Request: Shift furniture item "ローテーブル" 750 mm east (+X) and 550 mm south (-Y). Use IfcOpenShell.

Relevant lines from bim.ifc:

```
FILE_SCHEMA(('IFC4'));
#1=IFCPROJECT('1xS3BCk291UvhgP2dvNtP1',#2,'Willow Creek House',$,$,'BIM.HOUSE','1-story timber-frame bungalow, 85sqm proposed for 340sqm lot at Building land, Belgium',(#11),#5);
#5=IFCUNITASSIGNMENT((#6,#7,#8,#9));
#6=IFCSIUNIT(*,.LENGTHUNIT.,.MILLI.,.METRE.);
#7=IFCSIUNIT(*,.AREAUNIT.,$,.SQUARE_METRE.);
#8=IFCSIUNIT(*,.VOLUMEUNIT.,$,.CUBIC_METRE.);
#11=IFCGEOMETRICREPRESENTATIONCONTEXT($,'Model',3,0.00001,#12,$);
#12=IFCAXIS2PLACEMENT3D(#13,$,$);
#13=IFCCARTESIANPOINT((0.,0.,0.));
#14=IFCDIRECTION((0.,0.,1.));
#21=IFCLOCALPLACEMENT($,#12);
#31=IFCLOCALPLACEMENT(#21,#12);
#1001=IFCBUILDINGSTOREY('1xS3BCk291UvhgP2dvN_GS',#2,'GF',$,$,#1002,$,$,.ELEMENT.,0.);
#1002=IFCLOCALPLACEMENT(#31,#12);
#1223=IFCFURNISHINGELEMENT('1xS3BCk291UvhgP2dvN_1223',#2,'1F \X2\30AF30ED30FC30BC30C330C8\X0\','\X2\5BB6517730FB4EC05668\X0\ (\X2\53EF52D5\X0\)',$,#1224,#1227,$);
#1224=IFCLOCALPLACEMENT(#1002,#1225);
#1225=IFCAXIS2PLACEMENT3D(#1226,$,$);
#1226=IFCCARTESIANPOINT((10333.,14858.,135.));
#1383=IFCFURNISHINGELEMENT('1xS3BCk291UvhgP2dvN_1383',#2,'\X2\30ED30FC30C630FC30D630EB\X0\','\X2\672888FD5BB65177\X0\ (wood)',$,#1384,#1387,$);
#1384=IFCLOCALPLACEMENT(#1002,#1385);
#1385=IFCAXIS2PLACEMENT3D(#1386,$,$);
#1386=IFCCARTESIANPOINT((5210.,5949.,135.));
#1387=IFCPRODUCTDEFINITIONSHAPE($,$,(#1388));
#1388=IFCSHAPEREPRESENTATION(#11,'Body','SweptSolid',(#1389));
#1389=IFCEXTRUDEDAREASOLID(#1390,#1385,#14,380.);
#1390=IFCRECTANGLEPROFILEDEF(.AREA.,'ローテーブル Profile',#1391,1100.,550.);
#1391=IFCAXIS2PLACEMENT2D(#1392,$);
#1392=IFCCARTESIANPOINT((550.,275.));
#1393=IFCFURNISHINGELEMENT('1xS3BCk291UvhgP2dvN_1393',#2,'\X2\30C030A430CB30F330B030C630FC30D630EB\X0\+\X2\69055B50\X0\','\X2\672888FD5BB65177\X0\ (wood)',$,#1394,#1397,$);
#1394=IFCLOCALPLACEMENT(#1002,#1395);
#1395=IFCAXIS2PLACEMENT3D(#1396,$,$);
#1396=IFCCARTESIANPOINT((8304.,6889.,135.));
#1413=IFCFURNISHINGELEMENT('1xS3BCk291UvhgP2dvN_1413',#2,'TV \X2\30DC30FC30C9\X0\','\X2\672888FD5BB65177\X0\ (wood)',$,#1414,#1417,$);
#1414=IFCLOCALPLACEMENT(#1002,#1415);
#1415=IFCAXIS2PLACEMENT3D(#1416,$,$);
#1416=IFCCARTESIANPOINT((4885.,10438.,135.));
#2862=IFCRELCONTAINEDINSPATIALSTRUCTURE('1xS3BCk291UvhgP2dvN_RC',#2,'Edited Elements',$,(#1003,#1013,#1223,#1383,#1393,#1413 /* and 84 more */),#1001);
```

```python
import ifcopenshell
import ifcopenshell.api.geometry
import ifcopenshell.util.placement
import ifcopenshell.util.unit

model = ifcopenshell.open("bim.ifc")
unit_scale = ifcopenshell.util.unit.calculate_unit_scale(model)

item = model.by_id(1383)
matrix = ifcopenshell.util.placement.get_local_placement(item.ObjectPlacement)
matrix[0, 3] += 0.75 / unit_scale
matrix[1, 3] -= 0.55 / unit_scale
ifcopenshell.api.geometry.edit_object_placement(model, product=item, matrix=matrix, is_si=False)

print(ifcopenshell.util.placement.get_local_placement(item.ObjectPlacement).round(3) + 0.0)

model.write("bim_edited.ifc")
```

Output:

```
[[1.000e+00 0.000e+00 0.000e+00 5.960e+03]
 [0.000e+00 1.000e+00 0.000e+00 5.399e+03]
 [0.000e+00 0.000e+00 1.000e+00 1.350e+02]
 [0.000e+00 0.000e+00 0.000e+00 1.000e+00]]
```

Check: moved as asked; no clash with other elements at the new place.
